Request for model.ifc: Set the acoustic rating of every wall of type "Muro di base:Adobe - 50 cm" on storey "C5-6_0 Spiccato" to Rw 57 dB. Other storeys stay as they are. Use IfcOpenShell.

First a look at what the model holds.

```python
import ifcopenshell
import ifcopenshell.util.element

model = ifcopenshell.open("model.ifc")
print(model.schema)
storey = next(s for s in model.by_type("IfcBuildingStorey") if s.Name == "C5-6_0 Spiccato")
walls = [e for e in ifcopenshell.util.element.get_decomposition(storey) if e.is_a("IfcWall")]
seen = {}
for e in walls:
    element_type = ifcopenshell.util.element.get_type(e)
    key = (element_type.Name if element_type != e and element_type else None, ifcopenshell.util.element.get_pset(e, "Pset_WallCommon", "AcousticRating"))
    seen[key] = seen.get(key, 0) + 1
for (name, value), count in sorted(seen.items(), key=str):
    print(count, "x", name, "|", value)
```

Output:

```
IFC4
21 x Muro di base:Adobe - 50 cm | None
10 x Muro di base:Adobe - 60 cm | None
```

```python
import ifcopenshell
import ifcopenshell.api.pset
import ifcopenshell.util.element

model = ifcopenshell.open("model.ifc")

storey = next(s for s in model.by_type("IfcBuildingStorey") if s.Name == "C5-6_0 Spiccato")
walls = [e for e in ifcopenshell.util.element.get_decomposition(storey) if e.is_a("IfcWall")]

count = 0
for e in walls:
    element_type = ifcopenshell.util.element.get_type(e)
    if element_type in (None, e) or element_type.Name != "Muro di base:Adobe - 50 cm":
        continue
    # add_pset returns the element's existing set when there is one.
    pset = ifcopenshell.api.pset.add_pset(model, product=e, name="Pset_WallCommon")
    ifcopenshell.api.pset.edit_pset(model, pset=pset, properties={"AcousticRating": "Rw 57 dB"})
    count += 1

print(count, "walls updated")

model.write("model_v2.ifc")
```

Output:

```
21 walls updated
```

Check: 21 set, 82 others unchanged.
